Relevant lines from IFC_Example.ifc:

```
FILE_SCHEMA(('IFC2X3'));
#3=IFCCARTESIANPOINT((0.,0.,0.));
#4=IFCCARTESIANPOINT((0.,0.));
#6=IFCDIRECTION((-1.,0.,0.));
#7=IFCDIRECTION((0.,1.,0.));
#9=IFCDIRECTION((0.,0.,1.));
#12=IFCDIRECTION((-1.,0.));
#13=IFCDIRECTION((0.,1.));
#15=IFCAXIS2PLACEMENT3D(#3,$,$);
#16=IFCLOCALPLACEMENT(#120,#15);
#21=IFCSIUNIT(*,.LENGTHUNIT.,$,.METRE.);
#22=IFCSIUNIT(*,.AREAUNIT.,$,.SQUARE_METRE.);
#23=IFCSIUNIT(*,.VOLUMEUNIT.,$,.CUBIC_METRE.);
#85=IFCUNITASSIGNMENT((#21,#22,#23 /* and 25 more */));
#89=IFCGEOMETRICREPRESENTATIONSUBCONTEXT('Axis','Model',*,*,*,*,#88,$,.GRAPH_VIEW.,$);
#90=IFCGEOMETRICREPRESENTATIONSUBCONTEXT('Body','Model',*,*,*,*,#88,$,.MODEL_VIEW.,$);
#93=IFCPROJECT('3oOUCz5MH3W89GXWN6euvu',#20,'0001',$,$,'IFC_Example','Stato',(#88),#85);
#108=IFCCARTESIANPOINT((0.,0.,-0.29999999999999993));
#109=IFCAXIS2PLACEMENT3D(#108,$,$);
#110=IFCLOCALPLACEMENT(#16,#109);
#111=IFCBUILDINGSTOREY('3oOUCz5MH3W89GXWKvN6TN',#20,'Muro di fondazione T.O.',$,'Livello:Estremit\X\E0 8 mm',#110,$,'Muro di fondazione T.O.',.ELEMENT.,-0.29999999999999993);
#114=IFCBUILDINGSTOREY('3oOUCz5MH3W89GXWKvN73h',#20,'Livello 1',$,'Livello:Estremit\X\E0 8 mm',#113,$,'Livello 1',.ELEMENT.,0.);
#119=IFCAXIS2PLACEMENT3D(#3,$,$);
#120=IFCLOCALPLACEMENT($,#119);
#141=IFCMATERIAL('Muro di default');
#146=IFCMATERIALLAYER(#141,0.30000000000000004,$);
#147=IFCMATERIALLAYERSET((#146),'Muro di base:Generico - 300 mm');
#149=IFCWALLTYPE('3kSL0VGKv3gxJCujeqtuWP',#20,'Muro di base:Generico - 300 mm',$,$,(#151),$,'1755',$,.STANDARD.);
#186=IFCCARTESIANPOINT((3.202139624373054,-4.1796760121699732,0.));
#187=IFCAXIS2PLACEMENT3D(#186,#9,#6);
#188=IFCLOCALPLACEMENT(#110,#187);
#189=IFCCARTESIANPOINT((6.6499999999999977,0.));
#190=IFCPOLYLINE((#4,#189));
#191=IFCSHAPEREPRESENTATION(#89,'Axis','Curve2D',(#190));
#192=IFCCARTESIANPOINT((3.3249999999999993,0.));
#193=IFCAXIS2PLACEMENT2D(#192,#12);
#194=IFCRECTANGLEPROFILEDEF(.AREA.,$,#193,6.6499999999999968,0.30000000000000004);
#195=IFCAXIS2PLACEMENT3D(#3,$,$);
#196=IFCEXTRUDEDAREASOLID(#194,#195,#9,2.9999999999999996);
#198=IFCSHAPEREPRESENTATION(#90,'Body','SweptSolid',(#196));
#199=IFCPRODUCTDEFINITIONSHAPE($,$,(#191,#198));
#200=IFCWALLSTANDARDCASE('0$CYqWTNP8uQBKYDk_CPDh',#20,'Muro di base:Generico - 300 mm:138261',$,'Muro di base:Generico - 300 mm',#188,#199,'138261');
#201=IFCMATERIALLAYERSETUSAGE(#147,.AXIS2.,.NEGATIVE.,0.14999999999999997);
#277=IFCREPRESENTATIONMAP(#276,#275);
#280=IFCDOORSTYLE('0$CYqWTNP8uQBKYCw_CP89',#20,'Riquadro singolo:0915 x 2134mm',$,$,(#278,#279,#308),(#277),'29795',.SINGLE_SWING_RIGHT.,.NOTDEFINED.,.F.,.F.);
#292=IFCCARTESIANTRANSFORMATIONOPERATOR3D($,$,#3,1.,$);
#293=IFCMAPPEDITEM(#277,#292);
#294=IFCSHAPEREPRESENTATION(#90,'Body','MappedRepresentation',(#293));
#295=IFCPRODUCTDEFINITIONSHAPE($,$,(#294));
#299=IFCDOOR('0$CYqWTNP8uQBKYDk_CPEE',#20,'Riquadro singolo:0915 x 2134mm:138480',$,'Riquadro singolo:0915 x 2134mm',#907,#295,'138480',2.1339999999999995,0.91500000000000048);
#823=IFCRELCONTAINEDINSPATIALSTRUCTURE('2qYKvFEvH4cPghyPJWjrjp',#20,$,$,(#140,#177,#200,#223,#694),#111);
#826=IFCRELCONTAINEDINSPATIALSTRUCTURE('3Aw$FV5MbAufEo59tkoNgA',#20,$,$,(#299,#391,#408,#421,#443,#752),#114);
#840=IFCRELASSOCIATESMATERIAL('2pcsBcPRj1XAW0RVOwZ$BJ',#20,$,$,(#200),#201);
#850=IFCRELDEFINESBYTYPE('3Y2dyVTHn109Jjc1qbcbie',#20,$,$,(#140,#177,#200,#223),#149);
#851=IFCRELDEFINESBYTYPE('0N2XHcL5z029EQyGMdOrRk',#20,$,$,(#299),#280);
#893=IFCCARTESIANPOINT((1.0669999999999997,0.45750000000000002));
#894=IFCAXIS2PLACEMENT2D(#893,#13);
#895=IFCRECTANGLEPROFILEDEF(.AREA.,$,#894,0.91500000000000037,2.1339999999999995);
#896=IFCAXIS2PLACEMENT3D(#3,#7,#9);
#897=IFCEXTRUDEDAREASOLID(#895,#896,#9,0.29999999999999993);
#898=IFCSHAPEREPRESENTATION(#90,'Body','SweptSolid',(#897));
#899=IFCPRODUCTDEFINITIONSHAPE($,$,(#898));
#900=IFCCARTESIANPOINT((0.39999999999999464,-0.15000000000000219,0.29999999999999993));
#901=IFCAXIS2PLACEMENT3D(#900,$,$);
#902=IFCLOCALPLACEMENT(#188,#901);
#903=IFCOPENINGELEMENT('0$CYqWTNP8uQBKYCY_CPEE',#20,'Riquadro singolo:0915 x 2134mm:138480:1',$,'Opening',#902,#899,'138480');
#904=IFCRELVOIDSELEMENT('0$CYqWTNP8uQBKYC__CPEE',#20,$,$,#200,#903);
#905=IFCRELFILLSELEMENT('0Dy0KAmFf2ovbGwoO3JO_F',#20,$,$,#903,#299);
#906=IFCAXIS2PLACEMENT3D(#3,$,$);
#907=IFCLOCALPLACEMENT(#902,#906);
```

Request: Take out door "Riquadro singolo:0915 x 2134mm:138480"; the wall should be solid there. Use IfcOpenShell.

```python
import ifcopenshell
import ifcopenshell.api.feature
import ifcopenshell.api.root
import ifcopenshell.geom
import ifcopenshell.util.shape

model = ifcopenshell.open("IFC_Example.ifc")
settings = ifcopenshell.geom.settings()


def volume(element):
    """Net volume in cubic metres, openings subtracted."""
    shape = ifcopenshell.geom.create_shape(settings, element)
    return ifcopenshell.util.shape.get_volume(shape.geometry)


door = model.by_id(299)
opening = door.FillsVoids[0].RelatingOpeningElement
wall = opening.VoidsElements[0].RelatingBuildingElement
before = volume(wall)

ifcopenshell.api.root.remove_product(model, product=door)
ifcopenshell.api.feature.remove_feature(model, feature=opening)

after = volume(wall)

print(f"wall volume {before:.3f} -> {after:.3f} m3")

model.write("IFC_Example-out.ifc")
```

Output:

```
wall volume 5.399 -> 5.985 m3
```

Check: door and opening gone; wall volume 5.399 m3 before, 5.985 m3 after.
